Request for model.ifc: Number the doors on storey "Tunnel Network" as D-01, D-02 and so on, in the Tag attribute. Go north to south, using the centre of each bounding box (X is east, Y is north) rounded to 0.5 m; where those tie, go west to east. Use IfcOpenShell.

First a look at what the model holds.

```python
import ifcopenshell
import ifcopenshell.util.element
import ifcopenshell.util.placement

model = ifcopenshell.open("model.ifc")
print(model.schema)
storey = next(s for s in model.by_type("IfcBuildingStorey") if s.Name == "Tunnel Network")
doors = [e for e in ifcopenshell.util.element.get_decomposition(storey) if e.is_a("IfcDoor")]
for e in sorted(doors, key=lambda e: e.id()):
    origin = ifcopenshell.util.placement.get_local_placement(e.ObjectPlacement)[:3, 3]
    print(e.id(), e.Tag, e.Name, origin.round(2) + 0.0, sep=" | ")
```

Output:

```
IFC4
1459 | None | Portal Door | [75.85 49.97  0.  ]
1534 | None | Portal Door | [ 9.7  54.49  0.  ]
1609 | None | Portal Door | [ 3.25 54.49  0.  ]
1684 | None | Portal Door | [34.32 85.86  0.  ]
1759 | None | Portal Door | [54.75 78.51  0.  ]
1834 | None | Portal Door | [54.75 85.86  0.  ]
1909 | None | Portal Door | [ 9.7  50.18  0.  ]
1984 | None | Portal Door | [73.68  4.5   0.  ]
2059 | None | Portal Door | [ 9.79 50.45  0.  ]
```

```python
import ifcopenshell
import ifcopenshell.geom
import ifcopenshell.util.element
import ifcopenshell.util.shape

model = ifcopenshell.open("model.ifc")
settings = ifcopenshell.geom.settings()
settings.set("use-world-coords", True)


def centre(element):
    shape = ifcopenshell.geom.create_shape(settings, element)
    return ifcopenshell.util.shape.get_bbox_centroid(shape.geometry)


storey = next(s for s in model.by_type("IfcBuildingStorey") if s.Name == "Tunnel Network")
doors = [e for e in ifcopenshell.util.element.get_decomposition(storey) if e.is_a("IfcDoor")]

# Insertion points can sit at a corner or the storey origin, so sort by the geometry (in metres).
centres = {e: centre(e) for e in doors}
doors.sort(key=lambda e: (-round(centres[e][1] / 0.5), centres[e][0]))

for i, e in enumerate(doors, start=1):
    number = f"D-{i:02d}"
    e.Tag = number
    print(e.id(), number)

model.write("model_rev.ifc")
```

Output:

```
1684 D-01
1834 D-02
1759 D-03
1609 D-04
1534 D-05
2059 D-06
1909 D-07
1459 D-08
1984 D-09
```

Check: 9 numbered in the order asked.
